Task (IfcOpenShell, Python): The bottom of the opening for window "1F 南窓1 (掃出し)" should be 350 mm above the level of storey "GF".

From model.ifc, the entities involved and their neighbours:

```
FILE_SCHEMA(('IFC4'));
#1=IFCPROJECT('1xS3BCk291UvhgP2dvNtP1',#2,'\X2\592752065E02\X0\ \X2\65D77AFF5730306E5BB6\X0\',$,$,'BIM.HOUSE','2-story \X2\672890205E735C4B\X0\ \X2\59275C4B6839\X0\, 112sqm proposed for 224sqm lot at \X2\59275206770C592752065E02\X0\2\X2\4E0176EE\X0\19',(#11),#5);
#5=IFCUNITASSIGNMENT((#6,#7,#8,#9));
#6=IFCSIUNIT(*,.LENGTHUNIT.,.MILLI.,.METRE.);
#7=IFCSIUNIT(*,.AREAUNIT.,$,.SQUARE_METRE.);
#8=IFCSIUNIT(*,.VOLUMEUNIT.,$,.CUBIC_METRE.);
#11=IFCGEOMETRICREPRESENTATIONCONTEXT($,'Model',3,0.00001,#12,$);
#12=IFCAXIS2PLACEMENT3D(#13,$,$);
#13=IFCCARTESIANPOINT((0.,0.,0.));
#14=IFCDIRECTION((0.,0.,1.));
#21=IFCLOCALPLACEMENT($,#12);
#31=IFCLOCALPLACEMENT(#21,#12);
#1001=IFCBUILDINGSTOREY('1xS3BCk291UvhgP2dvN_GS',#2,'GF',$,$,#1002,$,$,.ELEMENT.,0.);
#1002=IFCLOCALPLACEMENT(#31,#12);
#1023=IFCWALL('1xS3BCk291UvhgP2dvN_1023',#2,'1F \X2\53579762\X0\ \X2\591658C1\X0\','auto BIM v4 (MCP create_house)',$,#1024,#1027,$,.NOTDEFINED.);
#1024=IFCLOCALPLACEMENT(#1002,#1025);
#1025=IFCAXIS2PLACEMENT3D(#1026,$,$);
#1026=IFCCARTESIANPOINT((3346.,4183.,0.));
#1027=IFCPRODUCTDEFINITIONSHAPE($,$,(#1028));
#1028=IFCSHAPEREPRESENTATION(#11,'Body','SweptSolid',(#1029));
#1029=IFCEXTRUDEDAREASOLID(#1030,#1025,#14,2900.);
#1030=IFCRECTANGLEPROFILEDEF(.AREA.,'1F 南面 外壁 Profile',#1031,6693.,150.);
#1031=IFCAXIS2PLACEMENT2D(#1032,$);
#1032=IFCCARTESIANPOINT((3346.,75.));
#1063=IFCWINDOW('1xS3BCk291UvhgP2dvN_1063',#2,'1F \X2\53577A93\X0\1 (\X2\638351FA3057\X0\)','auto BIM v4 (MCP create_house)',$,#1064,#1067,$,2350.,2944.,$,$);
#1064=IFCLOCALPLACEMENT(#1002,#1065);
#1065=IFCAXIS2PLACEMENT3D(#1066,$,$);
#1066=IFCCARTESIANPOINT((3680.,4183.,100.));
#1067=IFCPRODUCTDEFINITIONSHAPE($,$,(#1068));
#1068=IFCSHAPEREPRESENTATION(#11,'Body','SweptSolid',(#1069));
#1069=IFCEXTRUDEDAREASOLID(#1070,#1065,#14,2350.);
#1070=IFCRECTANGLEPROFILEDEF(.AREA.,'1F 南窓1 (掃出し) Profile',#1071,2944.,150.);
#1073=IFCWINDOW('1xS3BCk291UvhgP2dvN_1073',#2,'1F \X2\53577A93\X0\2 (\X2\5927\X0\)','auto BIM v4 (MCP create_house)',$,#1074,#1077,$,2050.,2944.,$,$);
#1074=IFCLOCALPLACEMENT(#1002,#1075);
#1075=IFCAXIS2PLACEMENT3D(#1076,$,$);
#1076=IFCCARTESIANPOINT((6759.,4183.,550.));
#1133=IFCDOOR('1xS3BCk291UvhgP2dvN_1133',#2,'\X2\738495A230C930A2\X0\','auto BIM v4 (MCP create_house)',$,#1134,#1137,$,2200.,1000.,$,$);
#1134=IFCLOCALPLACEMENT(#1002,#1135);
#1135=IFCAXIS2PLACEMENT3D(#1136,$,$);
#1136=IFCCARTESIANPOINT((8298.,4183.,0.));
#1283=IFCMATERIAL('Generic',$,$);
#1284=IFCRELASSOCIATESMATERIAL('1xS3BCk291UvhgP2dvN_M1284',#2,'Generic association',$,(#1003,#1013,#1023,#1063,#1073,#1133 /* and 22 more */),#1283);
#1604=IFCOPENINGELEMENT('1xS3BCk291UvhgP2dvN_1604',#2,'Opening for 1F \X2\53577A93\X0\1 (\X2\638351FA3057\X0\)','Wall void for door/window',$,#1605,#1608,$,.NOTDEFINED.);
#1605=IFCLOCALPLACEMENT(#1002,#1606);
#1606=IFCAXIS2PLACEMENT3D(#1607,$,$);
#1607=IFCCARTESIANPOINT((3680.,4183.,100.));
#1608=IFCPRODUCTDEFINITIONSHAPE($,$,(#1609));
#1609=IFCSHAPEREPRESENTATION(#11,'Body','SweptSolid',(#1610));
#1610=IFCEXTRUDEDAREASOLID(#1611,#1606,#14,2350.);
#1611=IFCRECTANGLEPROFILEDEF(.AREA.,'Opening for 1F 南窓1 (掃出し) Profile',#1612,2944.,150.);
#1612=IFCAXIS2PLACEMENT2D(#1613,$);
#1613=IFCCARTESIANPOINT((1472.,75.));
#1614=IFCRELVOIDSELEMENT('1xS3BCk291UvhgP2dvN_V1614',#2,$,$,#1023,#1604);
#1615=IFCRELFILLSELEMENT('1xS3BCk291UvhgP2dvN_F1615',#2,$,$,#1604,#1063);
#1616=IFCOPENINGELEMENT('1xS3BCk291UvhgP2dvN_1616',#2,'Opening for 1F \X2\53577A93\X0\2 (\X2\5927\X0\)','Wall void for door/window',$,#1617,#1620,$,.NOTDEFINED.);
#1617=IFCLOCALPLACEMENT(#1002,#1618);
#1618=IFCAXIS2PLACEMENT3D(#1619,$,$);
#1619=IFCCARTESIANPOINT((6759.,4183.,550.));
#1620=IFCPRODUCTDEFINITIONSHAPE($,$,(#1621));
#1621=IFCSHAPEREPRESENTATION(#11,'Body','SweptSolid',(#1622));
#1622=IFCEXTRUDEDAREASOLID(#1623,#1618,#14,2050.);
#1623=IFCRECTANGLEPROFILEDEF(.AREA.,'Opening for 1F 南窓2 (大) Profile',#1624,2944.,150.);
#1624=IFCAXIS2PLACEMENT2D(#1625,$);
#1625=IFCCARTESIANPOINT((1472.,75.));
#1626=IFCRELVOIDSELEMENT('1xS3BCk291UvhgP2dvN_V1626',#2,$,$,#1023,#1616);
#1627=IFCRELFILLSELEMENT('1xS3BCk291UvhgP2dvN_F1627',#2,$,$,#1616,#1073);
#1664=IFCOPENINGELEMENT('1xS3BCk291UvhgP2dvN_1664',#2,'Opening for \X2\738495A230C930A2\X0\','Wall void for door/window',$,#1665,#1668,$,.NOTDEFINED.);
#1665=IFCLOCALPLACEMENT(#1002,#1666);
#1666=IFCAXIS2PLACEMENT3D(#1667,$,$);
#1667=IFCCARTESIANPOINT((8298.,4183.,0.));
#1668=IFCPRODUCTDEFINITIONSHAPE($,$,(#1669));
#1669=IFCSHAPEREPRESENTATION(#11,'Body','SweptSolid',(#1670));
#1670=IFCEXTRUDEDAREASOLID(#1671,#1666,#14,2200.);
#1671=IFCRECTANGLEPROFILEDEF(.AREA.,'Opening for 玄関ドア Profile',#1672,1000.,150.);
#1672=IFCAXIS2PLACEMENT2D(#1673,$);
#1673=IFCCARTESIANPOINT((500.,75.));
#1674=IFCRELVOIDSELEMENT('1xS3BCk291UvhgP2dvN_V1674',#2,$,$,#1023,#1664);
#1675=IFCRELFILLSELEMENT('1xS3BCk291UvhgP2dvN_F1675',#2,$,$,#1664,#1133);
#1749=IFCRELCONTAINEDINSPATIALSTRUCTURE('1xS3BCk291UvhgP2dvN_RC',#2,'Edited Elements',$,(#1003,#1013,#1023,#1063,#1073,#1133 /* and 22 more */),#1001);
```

```python
import numpy as np
import ifcopenshell
import ifcopenshell.api.geometry
import ifcopenshell.geom
import ifcopenshell.util.element
import ifcopenshell.util.placement
import ifcopenshell.util.shape
import ifcopenshell.util.unit

model = ifcopenshell.open("model.ifc")
unit_scale = ifcopenshell.util.unit.calculate_unit_scale(model)

window = model.by_guid("1xS3BCk291UvhgP2dvN_1063")
opening = window.FillsVoids[0].RelatingOpeningElement
storey = ifcopenshell.util.element.get_container(window, ifc_class="IfcBuildingStorey")
level = ifcopenshell.util.placement.get_local_placement(storey.ObjectPlacement)[2, 3]

# The opening's origin need not be at the sill, so measure its lowest point.
shape = ifcopenshell.geom.create_shape(ifcopenshell.geom.settings(), opening)
bottom = ifcopenshell.util.shape.get_shape_bottom_elevation(shape, shape.geometry) / unit_scale
dz = level + 350.0 - bottom

shift = np.array([0.0, 0.0, dz])
# The window is not placed relative to its opening, so move both.
for product in (opening, window):
    matrix = ifcopenshell.util.placement.get_local_placement(product.ObjectPlacement)
    matrix[:3, 3] += shift
    ifcopenshell.api.geometry.edit_object_placement(model, product=product, matrix=matrix, is_si=False)

print(f"moved by {dz * unit_scale:+.3f} m")

model.write("model_edited.ifc")
```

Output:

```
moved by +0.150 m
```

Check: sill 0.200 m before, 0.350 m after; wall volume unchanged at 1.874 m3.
